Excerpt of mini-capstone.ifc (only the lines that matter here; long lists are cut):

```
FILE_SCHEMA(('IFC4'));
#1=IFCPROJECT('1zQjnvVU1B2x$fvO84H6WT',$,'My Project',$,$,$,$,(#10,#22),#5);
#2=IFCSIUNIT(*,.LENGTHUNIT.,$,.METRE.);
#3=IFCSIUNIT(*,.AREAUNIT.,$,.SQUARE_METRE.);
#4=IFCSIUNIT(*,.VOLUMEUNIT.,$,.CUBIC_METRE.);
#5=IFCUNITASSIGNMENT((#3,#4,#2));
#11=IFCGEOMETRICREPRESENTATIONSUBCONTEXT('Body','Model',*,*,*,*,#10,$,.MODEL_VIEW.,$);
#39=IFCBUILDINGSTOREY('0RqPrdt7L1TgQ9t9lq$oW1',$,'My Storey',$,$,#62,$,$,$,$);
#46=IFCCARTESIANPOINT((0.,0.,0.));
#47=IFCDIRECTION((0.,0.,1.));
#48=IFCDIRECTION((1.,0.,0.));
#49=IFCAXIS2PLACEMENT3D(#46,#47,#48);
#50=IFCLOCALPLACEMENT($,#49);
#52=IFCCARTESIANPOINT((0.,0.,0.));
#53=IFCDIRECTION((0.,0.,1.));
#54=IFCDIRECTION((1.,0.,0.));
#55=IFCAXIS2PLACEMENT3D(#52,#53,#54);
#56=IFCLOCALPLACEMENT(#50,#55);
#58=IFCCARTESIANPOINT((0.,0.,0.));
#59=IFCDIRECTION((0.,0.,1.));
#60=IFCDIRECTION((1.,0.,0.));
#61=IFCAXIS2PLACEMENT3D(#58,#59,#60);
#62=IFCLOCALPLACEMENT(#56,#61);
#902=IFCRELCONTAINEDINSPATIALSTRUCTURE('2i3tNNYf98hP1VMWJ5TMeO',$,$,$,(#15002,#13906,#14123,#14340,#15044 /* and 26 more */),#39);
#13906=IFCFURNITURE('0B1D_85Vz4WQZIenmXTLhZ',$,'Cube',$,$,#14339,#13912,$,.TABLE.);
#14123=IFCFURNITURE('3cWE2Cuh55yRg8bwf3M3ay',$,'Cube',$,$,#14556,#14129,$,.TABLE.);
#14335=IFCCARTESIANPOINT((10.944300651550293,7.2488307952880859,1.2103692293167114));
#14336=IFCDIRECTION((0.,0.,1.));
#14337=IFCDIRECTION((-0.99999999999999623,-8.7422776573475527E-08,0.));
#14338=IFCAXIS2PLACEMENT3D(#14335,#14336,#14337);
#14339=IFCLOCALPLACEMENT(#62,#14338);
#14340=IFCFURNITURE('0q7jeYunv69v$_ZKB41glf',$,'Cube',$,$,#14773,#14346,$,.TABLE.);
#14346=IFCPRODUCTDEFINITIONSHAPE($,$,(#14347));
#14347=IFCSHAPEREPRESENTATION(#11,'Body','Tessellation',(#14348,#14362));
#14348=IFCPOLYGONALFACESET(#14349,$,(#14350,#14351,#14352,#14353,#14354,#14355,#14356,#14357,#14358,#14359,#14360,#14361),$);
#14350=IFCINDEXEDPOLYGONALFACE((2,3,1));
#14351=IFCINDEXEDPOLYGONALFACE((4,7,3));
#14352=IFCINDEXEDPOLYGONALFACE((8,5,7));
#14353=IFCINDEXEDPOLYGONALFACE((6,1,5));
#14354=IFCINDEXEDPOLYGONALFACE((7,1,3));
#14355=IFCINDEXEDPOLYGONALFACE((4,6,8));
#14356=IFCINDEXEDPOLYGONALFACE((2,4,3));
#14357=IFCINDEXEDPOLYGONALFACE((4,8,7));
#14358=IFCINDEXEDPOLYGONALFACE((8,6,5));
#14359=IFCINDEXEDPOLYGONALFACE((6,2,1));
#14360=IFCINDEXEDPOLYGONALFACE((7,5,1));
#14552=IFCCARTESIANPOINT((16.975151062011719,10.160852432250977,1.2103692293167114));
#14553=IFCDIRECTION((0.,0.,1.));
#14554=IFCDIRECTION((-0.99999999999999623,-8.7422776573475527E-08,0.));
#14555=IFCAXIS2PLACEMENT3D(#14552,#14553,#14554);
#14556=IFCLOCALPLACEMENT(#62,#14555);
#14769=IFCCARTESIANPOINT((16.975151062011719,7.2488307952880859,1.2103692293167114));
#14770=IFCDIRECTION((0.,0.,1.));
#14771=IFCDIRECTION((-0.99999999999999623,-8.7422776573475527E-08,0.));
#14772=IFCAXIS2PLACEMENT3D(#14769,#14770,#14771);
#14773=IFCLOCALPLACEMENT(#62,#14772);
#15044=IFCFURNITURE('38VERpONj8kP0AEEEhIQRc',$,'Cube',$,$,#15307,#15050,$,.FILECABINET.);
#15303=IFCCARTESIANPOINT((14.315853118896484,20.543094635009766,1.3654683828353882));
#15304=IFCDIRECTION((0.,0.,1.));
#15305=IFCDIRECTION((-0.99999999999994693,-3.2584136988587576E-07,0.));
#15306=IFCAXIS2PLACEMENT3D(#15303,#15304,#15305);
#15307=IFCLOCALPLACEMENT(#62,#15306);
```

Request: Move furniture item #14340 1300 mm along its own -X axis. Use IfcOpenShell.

```python
import ifcopenshell
import ifcopenshell.api.geometry
import ifcopenshell.util.placement

model = ifcopenshell.open("mini-capstone.ifc")

item = model.by_id(14340)
matrix = ifcopenshell.util.placement.get_local_placement(item.ObjectPlacement)
matrix[:3, 3] -= matrix[:3, 0] * 1.3
ifcopenshell.api.geometry.edit_object_placement(model, product=item, matrix=matrix, is_si=False)

print(ifcopenshell.util.placement.get_local_placement(item.ObjectPlacement).round(3) + 0.0)

model.write("mini-capstone_rev.ifc")
```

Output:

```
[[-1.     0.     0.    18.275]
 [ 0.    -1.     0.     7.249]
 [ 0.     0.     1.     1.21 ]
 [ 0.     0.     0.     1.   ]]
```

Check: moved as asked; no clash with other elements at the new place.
